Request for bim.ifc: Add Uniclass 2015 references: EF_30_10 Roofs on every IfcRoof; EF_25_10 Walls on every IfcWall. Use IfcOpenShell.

First a look at what the model holds.

```python
import ifcopenshell

model = ifcopenshell.open("bim.ifc")
print(model.schema)
print("classifications:", [c.Name for c in model.by_type("IfcClassification")])
for ifc_class in ("IfcDoor", "IfcRoof", "IfcStair", "IfcWall", "IfcWindow"):
    print(ifc_class, len(model.by_type(ifc_class)))
```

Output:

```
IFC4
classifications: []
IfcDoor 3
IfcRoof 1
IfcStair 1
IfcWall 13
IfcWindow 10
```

```python
import ifcopenshell
import ifcopenshell.api.classification

model = ifcopenshell.open("bim.ifc")

system = ifcopenshell.api.classification.add_classification(model, classification="Uniclass 2015")

codes = {
    "IfcRoof": ("EF_30_10", "Roofs"),
    "IfcWall": ("EF_25_10", "Walls"),
}
for ifc_class, (code, name) in codes.items():
    products = model.by_type(ifc_class)
    ifcopenshell.api.classification.add_reference(
        model, products=products, classification=system, identification=code, name=name
    )
    print(code, len(products))

model.write("bim_updated.ifc")
```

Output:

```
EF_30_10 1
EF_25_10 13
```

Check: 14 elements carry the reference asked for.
